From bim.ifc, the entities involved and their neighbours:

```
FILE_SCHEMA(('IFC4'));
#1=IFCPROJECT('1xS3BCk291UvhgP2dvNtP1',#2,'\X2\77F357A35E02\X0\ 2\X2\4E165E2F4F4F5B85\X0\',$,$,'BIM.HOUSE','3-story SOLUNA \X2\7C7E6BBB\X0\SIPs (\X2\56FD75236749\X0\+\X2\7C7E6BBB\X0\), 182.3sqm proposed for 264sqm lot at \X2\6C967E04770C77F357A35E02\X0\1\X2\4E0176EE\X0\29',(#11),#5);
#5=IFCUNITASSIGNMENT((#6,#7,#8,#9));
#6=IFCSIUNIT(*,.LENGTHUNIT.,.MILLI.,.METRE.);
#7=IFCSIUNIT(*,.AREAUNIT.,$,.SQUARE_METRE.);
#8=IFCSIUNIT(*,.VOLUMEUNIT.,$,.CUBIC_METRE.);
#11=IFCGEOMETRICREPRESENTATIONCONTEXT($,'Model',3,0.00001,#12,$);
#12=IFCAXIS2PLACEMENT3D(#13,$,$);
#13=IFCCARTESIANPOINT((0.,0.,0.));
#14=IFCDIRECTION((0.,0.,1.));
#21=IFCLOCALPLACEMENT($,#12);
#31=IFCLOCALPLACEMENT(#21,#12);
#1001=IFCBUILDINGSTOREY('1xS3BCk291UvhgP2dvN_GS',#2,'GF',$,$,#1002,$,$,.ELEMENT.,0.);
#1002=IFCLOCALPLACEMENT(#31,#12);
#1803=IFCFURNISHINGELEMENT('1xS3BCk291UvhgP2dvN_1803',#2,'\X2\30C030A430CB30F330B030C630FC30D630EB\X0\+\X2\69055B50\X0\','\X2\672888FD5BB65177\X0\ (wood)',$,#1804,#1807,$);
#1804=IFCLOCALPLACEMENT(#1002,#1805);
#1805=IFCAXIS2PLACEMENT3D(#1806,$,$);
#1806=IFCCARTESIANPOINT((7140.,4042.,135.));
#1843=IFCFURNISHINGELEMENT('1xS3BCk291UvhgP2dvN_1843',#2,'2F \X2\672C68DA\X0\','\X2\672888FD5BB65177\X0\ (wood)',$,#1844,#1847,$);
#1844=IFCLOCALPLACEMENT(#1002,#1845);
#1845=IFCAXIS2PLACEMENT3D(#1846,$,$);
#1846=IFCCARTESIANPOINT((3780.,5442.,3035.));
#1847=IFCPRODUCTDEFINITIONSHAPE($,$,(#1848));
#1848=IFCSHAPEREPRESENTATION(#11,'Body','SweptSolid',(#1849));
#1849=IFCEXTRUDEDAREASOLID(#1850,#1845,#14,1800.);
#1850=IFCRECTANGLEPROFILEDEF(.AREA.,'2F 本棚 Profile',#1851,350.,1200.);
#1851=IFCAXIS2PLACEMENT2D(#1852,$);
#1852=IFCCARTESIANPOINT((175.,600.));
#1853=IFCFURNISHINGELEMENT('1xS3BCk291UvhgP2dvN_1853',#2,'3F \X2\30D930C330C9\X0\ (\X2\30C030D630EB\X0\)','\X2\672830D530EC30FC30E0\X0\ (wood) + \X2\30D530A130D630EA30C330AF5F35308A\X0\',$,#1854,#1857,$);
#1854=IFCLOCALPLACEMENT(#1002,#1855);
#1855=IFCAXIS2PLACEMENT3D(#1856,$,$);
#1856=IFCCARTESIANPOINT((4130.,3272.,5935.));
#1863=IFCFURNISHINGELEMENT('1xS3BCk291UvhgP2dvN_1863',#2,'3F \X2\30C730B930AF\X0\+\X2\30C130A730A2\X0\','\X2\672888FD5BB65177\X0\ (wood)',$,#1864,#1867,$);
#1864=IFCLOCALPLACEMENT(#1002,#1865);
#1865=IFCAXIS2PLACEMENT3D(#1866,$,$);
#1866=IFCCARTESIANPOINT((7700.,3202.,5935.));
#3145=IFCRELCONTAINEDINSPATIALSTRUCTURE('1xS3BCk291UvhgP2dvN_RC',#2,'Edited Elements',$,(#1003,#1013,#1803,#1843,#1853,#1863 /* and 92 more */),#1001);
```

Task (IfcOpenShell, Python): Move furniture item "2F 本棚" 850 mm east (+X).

```python
import ifcopenshell
import ifcopenshell.api.geometry
import ifcopenshell.util.placement

model = ifcopenshell.open("bim.ifc")

item = model.by_id(1843)
matrix = ifcopenshell.util.placement.get_local_placement(item.ObjectPlacement)
matrix[0, 3] += 850.0
ifcopenshell.api.geometry.edit_object_placement(model, product=item, matrix=matrix, is_si=False)

print(ifcopenshell.util.placement.get_local_placement(item.ObjectPlacement).round(3) + 0.0)

model.write("bim-out.ifc")
```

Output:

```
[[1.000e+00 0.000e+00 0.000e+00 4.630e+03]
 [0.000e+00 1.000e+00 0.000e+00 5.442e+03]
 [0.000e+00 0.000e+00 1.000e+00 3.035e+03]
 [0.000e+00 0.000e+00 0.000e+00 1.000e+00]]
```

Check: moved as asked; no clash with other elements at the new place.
